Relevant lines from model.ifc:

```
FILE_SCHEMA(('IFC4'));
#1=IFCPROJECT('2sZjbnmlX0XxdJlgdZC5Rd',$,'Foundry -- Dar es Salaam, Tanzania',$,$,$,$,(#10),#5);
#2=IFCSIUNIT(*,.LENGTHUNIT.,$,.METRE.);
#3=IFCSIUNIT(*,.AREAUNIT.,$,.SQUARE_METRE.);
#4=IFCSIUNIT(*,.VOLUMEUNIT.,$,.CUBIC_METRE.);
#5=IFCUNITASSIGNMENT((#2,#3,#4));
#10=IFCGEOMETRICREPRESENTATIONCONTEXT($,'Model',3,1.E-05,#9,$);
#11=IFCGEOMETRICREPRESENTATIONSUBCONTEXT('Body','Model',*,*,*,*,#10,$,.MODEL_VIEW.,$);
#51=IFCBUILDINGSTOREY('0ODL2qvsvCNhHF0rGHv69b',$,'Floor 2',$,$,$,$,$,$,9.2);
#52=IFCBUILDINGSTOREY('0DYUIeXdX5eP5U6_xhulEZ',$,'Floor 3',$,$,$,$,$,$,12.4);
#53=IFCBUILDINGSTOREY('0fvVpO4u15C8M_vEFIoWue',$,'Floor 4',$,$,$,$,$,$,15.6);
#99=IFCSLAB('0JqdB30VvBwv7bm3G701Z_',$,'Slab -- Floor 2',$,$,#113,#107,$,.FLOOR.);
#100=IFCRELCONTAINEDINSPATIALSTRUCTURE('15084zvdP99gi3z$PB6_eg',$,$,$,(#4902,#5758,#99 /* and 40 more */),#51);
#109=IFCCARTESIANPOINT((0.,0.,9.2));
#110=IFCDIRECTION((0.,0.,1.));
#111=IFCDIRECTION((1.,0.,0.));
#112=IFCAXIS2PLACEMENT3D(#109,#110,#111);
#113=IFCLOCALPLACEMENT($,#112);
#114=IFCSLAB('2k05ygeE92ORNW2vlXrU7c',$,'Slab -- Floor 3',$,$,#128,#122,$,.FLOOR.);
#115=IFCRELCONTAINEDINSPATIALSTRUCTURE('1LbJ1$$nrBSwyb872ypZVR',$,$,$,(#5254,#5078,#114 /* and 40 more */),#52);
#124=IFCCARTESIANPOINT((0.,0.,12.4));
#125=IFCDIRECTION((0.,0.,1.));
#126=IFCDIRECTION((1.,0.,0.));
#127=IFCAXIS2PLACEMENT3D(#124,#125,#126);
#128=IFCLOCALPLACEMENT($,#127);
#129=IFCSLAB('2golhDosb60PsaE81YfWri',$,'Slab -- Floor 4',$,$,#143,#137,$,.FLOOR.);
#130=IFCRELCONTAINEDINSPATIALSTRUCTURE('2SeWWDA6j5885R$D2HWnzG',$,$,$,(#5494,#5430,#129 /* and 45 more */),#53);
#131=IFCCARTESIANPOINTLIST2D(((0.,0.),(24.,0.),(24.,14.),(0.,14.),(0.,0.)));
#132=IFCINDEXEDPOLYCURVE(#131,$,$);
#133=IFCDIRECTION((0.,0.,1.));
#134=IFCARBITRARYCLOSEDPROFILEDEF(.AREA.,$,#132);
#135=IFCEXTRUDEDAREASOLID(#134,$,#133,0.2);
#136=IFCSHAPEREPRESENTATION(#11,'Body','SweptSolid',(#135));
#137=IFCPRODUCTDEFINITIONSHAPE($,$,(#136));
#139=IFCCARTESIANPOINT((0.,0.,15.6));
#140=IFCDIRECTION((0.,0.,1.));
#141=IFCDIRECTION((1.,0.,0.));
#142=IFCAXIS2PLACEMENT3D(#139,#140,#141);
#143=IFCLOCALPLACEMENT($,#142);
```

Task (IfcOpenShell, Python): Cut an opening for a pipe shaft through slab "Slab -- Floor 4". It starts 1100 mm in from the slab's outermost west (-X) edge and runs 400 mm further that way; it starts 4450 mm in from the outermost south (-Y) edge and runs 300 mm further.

```python
import numpy as np
import ifcopenshell
import ifcopenshell.api.feature
import ifcopenshell.api.geometry
import ifcopenshell.api.root
import ifcopenshell.geom
import ifcopenshell.util.placement
import ifcopenshell.util.representation
import ifcopenshell.util.shape
import ifcopenshell.util.unit

model = ifcopenshell.open("model.ifc")
unit_scale = ifcopenshell.util.unit.calculate_unit_scale(model)
settings = ifcopenshell.geom.settings()


def volume(element):
    """Net volume in cubic metres, openings subtracted."""
    shape = ifcopenshell.geom.create_shape(settings, element)
    return ifcopenshell.util.shape.get_volume(shape.geometry)


slab = model.by_guid("2golhDosb60PsaE81YfWri")
before = volume(slab)

# Extent in the slab's own axes, in metres. The edges named are its -X and -Y sides.
slab_shape = ifcopenshell.geom.create_shape(settings, slab)
vertices = ifcopenshell.util.shape.get_vertices(slab_shape.geometry)
x_min, y_min, bottom = vertices.min(axis=0)
top = vertices[:, 2].max()

opening = ifcopenshell.api.root.create_entity(model, ifc_class="IfcOpeningElement", name="Pipe shaft opening", predefined_type="OPENING")
context = ifcopenshell.util.representation.get_context(model, "Model", "Body", "MODEL_VIEW")
width, depth = 0.4, 0.3
outline = [(0.0, 0.0), (width, 0.0), (width, depth), (0.0, depth), (0.0, 0.0)]
# Overshoot both faces by 50 mm so the cut is clean.
shape = ifcopenshell.api.geometry.add_slab_representation(
    model, context=context, depth=top - bottom + 0.1, polyline=outline
)
ifcopenshell.api.geometry.assign_representation(model, product=opening, representation=shape)

matrix = ifcopenshell.util.placement.get_local_placement(slab.ObjectPlacement)
matrix[:, 3] = matrix @ np.append(np.array([x_min + 1.1, y_min + 4.45, bottom - 0.05]) / unit_scale, 1.0)
ifcopenshell.api.geometry.edit_object_placement(model, product=opening, matrix=matrix, is_si=False)
ifcopenshell.api.feature.add_feature(model, feature=opening, element=slab)

after = volume(slab)

print(f"slab volume {before:.3f} -> {after:.3f} m3")

model.write("model_edited.ifc")
```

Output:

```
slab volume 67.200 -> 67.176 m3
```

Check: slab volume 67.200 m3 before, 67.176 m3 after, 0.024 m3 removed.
